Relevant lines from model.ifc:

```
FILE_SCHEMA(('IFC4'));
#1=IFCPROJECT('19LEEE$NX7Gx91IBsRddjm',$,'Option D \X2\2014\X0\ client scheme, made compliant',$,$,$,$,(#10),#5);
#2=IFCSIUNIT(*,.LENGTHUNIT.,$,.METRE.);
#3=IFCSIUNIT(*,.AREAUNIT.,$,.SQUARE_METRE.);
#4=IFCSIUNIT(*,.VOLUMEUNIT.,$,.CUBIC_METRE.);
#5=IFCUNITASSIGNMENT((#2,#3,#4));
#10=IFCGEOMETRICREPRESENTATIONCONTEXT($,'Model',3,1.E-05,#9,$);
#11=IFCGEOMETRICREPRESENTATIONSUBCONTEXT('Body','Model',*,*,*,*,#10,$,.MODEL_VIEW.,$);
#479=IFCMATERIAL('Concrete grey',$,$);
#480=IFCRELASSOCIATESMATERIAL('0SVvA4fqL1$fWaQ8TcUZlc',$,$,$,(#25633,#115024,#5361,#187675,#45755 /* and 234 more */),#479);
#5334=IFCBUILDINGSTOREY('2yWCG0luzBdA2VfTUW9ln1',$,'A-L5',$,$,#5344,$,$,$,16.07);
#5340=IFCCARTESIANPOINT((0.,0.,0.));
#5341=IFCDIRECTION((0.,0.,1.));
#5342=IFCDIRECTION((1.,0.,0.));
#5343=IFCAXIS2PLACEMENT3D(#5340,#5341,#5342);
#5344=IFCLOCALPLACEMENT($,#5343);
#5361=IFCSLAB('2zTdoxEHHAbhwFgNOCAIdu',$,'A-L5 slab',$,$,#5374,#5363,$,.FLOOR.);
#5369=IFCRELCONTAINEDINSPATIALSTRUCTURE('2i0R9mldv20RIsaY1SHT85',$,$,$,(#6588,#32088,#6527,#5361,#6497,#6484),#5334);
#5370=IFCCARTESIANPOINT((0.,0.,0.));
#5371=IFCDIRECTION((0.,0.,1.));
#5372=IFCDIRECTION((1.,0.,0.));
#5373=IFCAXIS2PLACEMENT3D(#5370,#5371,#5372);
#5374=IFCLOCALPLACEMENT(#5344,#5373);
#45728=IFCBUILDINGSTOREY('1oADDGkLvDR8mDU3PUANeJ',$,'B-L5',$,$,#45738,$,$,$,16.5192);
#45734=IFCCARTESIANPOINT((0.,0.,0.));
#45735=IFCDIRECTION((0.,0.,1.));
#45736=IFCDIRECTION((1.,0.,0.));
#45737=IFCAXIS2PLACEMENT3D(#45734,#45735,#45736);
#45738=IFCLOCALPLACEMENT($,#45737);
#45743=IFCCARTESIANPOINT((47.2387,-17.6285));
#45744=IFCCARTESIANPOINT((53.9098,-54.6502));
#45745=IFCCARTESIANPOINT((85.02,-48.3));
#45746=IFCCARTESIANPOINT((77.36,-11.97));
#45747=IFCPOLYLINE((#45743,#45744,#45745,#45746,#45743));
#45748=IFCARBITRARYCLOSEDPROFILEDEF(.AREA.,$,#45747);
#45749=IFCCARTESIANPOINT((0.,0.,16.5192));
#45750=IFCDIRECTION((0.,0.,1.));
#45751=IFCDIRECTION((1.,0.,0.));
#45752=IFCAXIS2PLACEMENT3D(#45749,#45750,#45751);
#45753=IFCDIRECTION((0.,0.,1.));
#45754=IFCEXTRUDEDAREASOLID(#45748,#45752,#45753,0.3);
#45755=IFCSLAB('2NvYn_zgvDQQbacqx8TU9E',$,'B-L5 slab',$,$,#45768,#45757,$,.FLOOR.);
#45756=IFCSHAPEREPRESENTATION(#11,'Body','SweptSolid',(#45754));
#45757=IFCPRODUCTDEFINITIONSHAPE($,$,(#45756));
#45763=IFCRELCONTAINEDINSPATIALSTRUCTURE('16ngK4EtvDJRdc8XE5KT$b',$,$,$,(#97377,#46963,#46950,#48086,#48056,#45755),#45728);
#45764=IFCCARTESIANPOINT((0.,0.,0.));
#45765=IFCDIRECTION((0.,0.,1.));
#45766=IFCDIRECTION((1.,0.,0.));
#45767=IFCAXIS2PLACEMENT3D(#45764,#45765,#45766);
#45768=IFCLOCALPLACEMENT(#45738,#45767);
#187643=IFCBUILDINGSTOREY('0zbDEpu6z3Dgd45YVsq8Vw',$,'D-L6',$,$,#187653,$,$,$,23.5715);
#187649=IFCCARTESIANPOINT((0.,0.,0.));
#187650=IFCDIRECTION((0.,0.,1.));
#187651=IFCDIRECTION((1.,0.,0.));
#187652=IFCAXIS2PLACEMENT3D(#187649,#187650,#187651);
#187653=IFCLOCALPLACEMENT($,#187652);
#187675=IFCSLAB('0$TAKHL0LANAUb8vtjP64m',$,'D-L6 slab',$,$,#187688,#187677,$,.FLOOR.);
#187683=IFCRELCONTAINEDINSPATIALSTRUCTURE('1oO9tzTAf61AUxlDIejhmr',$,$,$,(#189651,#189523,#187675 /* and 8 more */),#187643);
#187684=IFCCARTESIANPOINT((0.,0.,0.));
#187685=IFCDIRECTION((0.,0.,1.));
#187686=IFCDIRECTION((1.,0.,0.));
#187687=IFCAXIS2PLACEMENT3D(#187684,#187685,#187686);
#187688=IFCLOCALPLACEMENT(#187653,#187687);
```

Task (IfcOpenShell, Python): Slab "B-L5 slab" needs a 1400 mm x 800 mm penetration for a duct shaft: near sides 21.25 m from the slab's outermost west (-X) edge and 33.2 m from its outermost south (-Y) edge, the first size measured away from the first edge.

```python
import numpy as np
import ifcopenshell
import ifcopenshell.api.feature
import ifcopenshell.api.geometry
import ifcopenshell.api.root
import ifcopenshell.geom
import ifcopenshell.util.placement
import ifcopenshell.util.representation
import ifcopenshell.util.shape
import ifcopenshell.util.unit

model = ifcopenshell.open("model.ifc")
unit_scale = ifcopenshell.util.unit.calculate_unit_scale(model)
settings = ifcopenshell.geom.settings()


def volume(element):
    """Net volume in cubic metres, openings subtracted."""
    shape = ifcopenshell.geom.create_shape(settings, element)
    return ifcopenshell.util.shape.get_volume(shape.geometry)


slab = model.by_guid("2NvYn_zgvDQQbacqx8TU9E")
before = volume(slab)

# Extent in the slab's own axes, in metres. The edges named are its -X and -Y sides.
slab_shape = ifcopenshell.geom.create_shape(settings, slab)
vertices = ifcopenshell.util.shape.get_vertices(slab_shape.geometry)
x_min, y_min, bottom = vertices.min(axis=0)
top = vertices[:, 2].max()

opening = ifcopenshell.api.root.create_entity(model, ifc_class="IfcOpeningElement", name="Duct shaft opening", predefined_type="OPENING")
context = ifcopenshell.util.representation.get_context(model, "Model", "Body", "MODEL_VIEW")
width, depth = 1.4, 0.8
outline = [(0.0, 0.0), (width, 0.0), (width, depth), (0.0, depth), (0.0, 0.0)]
# Overshoot both faces by 50 mm so the cut is clean.
shape = ifcopenshell.api.geometry.add_slab_representation(
    model, context=context, depth=top - bottom + 0.1, polyline=outline
)
ifcopenshell.api.geometry.assign_representation(model, product=opening, representation=shape)

matrix = ifcopenshell.util.placement.get_local_placement(slab.ObjectPlacement)
matrix[:, 3] = matrix @ np.append(np.array([x_min + 21.25, y_min + 33.2, bottom - 0.05]) / unit_scale, 1.0)
ifcopenshell.api.geometry.edit_object_placement(model, product=opening, matrix=matrix, is_si=False)
ifcopenshell.api.feature.add_feature(model, feature=opening, element=slab)

after = volume(slab)

print(f"slab volume {before:.3f} -> {after:.3f} m3")

model.write("model_rev.ifc")
```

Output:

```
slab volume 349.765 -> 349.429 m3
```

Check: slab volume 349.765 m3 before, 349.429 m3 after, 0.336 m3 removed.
